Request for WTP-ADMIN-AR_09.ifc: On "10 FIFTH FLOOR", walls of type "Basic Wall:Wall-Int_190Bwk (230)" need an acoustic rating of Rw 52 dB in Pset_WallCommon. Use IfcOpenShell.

First a look at what the model holds.

```python
import ifcopenshell
import ifcopenshell.util.element

model = ifcopenshell.open("WTP-ADMIN-AR_09.ifc")
print(model.schema)
storey = next(s for s in model.by_type("IfcBuildingStorey") if s.Name == "10 FIFTH FLOOR")
walls = [e for e in ifcopenshell.util.element.get_decomposition(storey) if e.is_a("IfcWall")]
seen = {}
for e in walls:
    element_type = ifcopenshell.util.element.get_type(e)
    key = (element_type.Name if element_type != e and element_type else None, ifcopenshell.util.element.get_pset(e, "Pset_WallCommon", "AcousticRating"))
    seen[key] = seen.get(key, 0) + 1
for (name, value), count in sorted(seen.items(), key=str):
    print(count, "x", name, "|", value)
```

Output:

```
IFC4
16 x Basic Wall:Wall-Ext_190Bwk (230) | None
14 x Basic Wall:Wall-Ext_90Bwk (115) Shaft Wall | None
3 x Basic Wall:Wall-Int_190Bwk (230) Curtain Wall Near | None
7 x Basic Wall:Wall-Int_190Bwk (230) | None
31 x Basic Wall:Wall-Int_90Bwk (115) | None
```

```python
import ifcopenshell
import ifcopenshell.api.pset
import ifcopenshell.util.element

model = ifcopenshell.open("WTP-ADMIN-AR_09.ifc")

storey = next(s for s in model.by_type("IfcBuildingStorey") if s.Name == "10 FIFTH FLOOR")
walls = [e for e in ifcopenshell.util.element.get_decomposition(storey) if e.is_a("IfcWall")]

count = 0
for e in walls:
    element_type = ifcopenshell.util.element.get_type(e)
    if element_type in (None, e) or element_type.Name != "Basic Wall:Wall-Int_190Bwk (230)":
        continue
    # add_pset returns the element's existing set when there is one.
    pset = ifcopenshell.api.pset.add_pset(model, product=e, name="Pset_WallCommon")
    ifcopenshell.api.pset.edit_pset(model, pset=pset, properties={"AcousticRating": "Rw 52 dB"})
    count += 1

print(count, "walls updated")

model.write("WTP-ADMIN-AR_09_edited.ifc")
```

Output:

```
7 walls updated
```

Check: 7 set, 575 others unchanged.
